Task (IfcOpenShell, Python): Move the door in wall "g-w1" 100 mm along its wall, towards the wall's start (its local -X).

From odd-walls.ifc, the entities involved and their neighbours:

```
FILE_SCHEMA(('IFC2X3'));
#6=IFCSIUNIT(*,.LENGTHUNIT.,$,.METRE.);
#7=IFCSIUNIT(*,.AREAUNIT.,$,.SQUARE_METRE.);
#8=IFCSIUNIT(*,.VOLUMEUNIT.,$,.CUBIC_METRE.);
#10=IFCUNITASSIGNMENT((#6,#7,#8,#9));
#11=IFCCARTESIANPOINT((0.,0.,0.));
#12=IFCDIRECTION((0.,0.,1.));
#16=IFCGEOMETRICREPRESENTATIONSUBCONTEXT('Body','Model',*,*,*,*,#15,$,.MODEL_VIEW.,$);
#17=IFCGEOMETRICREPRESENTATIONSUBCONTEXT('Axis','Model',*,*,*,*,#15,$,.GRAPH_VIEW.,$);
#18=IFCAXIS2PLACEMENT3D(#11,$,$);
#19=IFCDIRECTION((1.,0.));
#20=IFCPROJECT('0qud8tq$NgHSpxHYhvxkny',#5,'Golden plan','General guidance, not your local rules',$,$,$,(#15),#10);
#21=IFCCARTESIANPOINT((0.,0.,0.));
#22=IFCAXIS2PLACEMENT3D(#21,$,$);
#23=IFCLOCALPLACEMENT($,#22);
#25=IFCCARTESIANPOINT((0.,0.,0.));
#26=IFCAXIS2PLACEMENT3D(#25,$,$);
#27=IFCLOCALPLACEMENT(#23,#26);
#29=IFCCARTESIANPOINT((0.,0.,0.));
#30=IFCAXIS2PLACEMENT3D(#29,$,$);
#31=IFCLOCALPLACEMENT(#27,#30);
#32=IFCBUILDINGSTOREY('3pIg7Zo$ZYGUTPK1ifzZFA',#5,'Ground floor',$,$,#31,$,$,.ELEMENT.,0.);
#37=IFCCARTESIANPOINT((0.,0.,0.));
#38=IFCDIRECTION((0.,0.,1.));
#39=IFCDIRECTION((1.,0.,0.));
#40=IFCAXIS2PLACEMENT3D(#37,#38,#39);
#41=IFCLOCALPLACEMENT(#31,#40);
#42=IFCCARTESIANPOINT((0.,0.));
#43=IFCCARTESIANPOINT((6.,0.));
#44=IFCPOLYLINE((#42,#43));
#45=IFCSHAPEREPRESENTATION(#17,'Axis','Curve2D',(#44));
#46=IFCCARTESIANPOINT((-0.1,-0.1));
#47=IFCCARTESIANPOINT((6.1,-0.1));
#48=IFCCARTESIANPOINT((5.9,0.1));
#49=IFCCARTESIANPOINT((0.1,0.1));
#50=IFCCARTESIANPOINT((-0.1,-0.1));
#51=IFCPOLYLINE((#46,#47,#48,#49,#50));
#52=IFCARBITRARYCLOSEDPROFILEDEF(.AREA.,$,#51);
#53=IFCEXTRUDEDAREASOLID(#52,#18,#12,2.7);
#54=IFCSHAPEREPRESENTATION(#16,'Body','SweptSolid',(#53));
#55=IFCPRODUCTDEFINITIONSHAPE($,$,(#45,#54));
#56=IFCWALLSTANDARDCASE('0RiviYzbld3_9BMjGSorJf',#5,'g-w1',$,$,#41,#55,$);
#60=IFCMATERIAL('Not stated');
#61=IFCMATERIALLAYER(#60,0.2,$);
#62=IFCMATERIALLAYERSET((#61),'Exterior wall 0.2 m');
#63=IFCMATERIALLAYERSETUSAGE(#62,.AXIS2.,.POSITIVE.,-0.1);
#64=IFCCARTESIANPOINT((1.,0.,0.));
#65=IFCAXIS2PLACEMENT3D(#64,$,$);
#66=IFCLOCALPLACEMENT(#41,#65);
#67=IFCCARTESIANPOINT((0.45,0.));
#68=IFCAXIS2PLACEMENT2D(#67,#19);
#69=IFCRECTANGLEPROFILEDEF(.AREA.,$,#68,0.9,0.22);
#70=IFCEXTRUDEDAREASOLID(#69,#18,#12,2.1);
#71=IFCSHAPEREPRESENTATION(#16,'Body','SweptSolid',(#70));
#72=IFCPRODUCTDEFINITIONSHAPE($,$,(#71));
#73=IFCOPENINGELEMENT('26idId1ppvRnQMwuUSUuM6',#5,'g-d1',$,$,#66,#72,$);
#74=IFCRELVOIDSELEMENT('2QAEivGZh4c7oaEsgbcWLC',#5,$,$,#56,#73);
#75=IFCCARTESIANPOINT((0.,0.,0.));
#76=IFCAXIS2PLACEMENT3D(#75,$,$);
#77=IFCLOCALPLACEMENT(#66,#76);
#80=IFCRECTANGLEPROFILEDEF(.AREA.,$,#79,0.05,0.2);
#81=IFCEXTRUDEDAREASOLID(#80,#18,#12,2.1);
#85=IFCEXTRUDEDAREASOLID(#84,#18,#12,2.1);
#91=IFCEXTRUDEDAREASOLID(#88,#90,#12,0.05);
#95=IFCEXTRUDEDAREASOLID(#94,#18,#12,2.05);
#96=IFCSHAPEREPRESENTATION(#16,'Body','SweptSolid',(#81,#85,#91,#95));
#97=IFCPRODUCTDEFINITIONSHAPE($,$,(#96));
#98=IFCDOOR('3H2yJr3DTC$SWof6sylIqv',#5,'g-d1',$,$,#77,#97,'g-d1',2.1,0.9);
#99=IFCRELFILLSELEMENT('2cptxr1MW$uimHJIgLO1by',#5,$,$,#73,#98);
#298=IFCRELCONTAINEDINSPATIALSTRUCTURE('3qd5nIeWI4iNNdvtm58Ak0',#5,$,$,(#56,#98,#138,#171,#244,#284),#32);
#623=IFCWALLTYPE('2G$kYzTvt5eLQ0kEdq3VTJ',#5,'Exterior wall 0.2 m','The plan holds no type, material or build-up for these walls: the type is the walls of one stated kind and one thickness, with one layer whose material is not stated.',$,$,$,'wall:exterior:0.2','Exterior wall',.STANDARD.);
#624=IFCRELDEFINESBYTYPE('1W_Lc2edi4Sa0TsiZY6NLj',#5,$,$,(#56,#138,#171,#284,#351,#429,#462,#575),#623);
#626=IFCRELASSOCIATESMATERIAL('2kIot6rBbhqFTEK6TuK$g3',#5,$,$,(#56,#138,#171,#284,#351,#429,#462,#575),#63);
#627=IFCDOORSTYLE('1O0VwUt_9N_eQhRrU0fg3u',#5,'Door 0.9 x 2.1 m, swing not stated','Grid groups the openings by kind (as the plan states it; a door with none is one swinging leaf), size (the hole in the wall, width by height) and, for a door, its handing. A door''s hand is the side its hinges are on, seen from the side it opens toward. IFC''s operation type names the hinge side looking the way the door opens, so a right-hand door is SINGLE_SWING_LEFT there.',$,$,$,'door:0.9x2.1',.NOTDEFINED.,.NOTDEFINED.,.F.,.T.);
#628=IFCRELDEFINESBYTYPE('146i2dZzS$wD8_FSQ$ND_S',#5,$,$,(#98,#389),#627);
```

```python
import ifcopenshell
import ifcopenshell.api.geometry
import ifcopenshell.util.placement
import ifcopenshell.util.unit

model = ifcopenshell.open("odd-walls.ifc")
unit_scale = ifcopenshell.util.unit.calculate_unit_scale(model)

door = model.by_id(98)
opening = door.FillsVoids[0].RelatingOpeningElement
wall = opening.VoidsElements[0].RelatingBuildingElement

wall_matrix = ifcopenshell.util.placement.get_local_placement(wall.ObjectPlacement)
shift = wall_matrix[:3, 0] * -0.1 / unit_scale
before = ifcopenshell.util.placement.get_local_placement(door.ObjectPlacement)[:3, 3].copy()

# The door is placed relative to its opening, so it follows when the opening moves.
matrix = ifcopenshell.util.placement.get_local_placement(opening.ObjectPlacement)
matrix[:3, 3] += shift
ifcopenshell.api.geometry.edit_object_placement(
    model, product=opening, matrix=matrix, is_si=False, should_transform_children=True
)

after = ifcopenshell.util.placement.get_local_placement(door.ObjectPlacement)[:3, 3]
print("door moved by", (after - before).round(3) + 0.0)

model.write("odd-walls_updated.ifc")
```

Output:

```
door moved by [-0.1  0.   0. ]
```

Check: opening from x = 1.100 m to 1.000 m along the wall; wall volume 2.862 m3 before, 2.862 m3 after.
